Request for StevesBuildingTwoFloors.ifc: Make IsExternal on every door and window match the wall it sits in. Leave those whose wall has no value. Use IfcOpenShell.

First a look at what the model holds.

```python
import ifcopenshell
import ifcopenshell.util.element

model = ifcopenshell.open("StevesBuildingTwoFloors.ifc")
print(model.schema)
seen = {}
for e in model.by_type("IfcDoor") + model.by_type("IfcWindow"):
    if not e.FillsVoids:
        continue
    host = e.FillsVoids[0].RelatingOpeningElement.VoidsElements[0].RelatingBuildingElement
    own = ifcopenshell.util.element.get_pset(e, f"Pset_{e.is_a()[3:].removesuffix('StandardCase')}Common", "IsExternal")
    wall = ifcopenshell.util.element.get_pset(host, "Pset_WallCommon", "IsExternal")
    seen[e.is_a(), own, wall] = seen.get((e.is_a(), own, wall), 0) + 1
for (cls, own, wall), count in sorted(seen.items(), key=str):
    print(count, cls, "IsExternal:", own, "| host wall:", wall)
```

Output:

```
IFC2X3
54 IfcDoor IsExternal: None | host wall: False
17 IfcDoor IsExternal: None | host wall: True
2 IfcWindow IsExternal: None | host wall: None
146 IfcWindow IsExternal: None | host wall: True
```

```python
import ifcopenshell
import ifcopenshell.api.pset
import ifcopenshell.util.element

model = ifcopenshell.open("StevesBuildingTwoFloors.ifc")

count = 0
for ifc_class, pset_name in (("IfcDoor", "Pset_DoorCommon"), ("IfcWindow", "Pset_WindowCommon")):
    for e in model.by_type(ifc_class):
        if not e.FillsVoids:
            continue
        host = e.FillsVoids[0].RelatingOpeningElement.VoidsElements[0].RelatingBuildingElement
        external = ifcopenshell.util.element.get_pset(host, "Pset_WallCommon", "IsExternal")
        if external is None or ifcopenshell.util.element.get_pset(e, pset_name, "IsExternal") == external:
            continue
        pset = ifcopenshell.api.pset.add_pset(model, product=e, name=pset_name)
        ifcopenshell.api.pset.edit_pset(model, pset=pset, properties={"IsExternal": external})
        count += 1

print(count, "updated")

model.write("StevesBuildingTwoFloors_updated.ifc")
```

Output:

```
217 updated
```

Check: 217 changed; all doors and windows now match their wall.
